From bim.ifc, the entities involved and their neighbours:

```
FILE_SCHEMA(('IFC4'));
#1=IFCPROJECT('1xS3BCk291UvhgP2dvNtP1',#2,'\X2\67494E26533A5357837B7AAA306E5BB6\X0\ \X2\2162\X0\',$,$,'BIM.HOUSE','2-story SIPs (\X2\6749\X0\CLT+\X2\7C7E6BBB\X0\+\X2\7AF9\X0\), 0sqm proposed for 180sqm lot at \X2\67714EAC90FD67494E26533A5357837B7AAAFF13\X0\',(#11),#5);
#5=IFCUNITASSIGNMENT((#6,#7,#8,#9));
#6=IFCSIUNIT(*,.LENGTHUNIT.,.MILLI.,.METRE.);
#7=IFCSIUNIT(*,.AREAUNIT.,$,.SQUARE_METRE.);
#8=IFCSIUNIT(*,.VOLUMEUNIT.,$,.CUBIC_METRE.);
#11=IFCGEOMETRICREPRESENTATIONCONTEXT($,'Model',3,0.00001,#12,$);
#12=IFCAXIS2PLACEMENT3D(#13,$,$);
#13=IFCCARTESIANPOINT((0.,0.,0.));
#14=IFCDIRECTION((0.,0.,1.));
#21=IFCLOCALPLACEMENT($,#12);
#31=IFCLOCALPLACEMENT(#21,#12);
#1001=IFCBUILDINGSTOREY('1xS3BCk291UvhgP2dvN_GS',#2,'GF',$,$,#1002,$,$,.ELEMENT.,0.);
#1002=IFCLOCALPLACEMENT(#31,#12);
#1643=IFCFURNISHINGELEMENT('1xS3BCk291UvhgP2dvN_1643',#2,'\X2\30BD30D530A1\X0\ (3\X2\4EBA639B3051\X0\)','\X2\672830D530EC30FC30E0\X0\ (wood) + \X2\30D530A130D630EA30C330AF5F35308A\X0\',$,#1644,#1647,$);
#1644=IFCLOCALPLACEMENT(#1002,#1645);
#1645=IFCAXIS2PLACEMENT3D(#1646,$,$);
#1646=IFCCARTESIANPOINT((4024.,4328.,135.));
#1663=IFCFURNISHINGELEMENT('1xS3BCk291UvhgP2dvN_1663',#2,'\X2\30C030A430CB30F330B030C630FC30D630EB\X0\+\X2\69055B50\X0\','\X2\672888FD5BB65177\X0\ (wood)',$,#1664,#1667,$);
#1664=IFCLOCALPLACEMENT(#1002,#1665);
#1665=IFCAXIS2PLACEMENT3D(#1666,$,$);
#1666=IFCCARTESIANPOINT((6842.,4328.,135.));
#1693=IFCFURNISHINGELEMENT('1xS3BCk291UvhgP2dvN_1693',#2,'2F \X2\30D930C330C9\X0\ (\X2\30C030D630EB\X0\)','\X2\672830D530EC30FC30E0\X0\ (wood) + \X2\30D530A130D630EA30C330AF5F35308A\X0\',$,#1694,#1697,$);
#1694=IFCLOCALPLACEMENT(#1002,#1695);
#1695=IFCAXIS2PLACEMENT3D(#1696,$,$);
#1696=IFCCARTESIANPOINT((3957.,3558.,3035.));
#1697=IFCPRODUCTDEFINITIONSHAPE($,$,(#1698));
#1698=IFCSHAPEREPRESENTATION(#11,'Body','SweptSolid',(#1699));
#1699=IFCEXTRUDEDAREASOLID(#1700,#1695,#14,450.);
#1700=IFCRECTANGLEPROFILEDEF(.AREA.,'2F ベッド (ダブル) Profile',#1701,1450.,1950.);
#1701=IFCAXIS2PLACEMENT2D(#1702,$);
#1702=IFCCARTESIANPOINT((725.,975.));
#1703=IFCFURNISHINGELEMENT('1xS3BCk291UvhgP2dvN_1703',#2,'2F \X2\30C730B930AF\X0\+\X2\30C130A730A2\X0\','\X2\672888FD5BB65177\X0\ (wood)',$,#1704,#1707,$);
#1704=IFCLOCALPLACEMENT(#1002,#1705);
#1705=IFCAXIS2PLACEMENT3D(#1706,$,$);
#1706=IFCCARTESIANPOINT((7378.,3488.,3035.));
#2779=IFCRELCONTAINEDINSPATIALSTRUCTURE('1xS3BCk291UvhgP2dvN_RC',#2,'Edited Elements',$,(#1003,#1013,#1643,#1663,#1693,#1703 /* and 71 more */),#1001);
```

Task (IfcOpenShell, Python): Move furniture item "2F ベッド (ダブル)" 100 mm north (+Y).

```python
import ifcopenshell
import ifcopenshell.api.geometry
import ifcopenshell.util.placement

model = ifcopenshell.open("bim.ifc")

item = model.by_guid("1xS3BCk291UvhgP2dvN_1693")
matrix = ifcopenshell.util.placement.get_local_placement(item.ObjectPlacement)
matrix[1, 3] += 100.0
ifcopenshell.api.geometry.edit_object_placement(model, product=item, matrix=matrix, is_si=False)

print(ifcopenshell.util.placement.get_local_placement(item.ObjectPlacement).round(3) + 0.0)

model.write("bim_v2.ifc")
```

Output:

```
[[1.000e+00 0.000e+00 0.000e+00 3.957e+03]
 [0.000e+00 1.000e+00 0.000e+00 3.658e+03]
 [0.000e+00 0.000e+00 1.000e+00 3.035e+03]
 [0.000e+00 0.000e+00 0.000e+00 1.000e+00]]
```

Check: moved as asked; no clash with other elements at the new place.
